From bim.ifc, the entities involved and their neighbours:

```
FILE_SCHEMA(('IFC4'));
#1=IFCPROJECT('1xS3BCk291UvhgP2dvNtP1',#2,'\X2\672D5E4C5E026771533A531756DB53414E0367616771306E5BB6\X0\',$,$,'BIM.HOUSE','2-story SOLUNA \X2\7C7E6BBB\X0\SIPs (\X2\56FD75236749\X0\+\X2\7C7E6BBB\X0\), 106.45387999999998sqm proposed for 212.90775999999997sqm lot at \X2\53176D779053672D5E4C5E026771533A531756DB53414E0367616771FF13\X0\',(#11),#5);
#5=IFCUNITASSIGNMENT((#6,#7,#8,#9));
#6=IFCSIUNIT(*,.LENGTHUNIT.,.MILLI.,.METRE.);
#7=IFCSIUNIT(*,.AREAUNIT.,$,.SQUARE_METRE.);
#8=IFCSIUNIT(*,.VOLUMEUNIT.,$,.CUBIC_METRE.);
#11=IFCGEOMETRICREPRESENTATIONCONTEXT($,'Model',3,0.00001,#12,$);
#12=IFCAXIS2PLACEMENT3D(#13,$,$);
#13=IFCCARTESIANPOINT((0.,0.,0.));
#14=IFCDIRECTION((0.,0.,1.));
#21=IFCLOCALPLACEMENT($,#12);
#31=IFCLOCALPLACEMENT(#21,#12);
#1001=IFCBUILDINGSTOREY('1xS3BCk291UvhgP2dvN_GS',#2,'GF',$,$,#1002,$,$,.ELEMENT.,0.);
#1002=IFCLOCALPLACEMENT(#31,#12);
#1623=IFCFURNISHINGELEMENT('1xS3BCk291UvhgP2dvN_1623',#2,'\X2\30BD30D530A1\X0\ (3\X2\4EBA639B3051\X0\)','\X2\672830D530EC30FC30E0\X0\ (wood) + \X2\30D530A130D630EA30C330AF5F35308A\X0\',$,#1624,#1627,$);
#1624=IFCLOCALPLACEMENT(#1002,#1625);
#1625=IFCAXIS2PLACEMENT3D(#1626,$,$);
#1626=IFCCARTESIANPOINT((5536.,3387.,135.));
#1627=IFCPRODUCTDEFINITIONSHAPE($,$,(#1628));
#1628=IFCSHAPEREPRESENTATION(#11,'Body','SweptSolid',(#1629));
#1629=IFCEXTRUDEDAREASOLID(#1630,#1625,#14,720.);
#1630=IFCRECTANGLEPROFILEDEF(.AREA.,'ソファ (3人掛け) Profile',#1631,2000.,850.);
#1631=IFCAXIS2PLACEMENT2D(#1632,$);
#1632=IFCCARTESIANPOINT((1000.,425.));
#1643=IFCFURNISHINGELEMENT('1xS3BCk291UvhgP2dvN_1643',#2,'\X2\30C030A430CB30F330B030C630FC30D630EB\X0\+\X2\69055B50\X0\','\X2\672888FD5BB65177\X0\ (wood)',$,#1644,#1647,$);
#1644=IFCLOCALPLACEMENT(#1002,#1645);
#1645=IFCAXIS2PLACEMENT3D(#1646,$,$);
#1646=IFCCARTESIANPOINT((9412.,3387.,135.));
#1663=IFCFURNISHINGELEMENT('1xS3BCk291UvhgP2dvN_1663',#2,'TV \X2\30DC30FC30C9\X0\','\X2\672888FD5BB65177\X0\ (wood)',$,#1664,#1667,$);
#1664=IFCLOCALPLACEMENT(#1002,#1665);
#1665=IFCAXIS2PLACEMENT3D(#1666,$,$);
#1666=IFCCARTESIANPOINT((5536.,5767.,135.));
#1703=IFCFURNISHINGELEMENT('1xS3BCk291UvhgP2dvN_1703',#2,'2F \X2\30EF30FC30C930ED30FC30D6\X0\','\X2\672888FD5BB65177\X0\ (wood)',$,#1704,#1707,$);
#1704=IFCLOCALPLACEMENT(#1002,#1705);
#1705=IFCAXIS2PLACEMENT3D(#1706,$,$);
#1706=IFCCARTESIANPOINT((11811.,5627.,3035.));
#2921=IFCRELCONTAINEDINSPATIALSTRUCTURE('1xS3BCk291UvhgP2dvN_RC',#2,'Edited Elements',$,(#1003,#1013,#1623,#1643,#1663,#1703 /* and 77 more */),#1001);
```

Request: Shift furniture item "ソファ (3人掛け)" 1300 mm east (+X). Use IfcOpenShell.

```python
import ifcopenshell
import ifcopenshell.api.geometry
import ifcopenshell.util.placement
import ifcopenshell.util.unit

model = ifcopenshell.open("bim.ifc")
unit_scale = ifcopenshell.util.unit.calculate_unit_scale(model)

item = model.by_guid("1xS3BCk291UvhgP2dvN_1623")
matrix = ifcopenshell.util.placement.get_local_placement(item.ObjectPlacement)
matrix[0, 3] += 1.3 / unit_scale
ifcopenshell.api.geometry.edit_object_placement(model, product=item, matrix=matrix, is_si=False)

print(ifcopenshell.util.placement.get_local_placement(item.ObjectPlacement).round(3) + 0.0)

model.write("bim_edited.ifc")
```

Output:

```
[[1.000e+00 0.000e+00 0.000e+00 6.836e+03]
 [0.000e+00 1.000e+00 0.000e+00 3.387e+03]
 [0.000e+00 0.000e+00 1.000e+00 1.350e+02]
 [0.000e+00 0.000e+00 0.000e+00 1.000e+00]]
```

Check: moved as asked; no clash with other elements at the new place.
